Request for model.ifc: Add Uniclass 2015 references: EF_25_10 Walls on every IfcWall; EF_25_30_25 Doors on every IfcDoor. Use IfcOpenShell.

First a look at what the model holds.

```python
import ifcopenshell

model = ifcopenshell.open("model.ifc")
print(model.schema)
print("classifications:", [c.Name for c in model.by_type("IfcClassification")])
for ifc_class in ("IfcDoor", "IfcRoof", "IfcStair", "IfcWall", "IfcWindow"):
    print(ifc_class, len(model.by_type(ifc_class)))
```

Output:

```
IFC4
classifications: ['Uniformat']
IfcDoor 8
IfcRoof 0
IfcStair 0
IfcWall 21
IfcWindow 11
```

```python
import ifcopenshell
import ifcopenshell.api.classification

model = ifcopenshell.open("model.ifc")

system = ifcopenshell.api.classification.add_classification(model, classification="Uniclass 2015")

codes = {
    "IfcWall": ("EF_25_10", "Walls"),
    "IfcDoor": ("EF_25_30_25", "Doors"),
}
for ifc_class, (code, name) in codes.items():
    products = model.by_type(ifc_class)
    ifcopenshell.api.classification.add_reference(
        model, products=products, classification=system, identification=code, name=name
    )
    print(code, len(products))

model.write("model-out.ifc")
```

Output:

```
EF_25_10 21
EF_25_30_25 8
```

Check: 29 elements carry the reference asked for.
